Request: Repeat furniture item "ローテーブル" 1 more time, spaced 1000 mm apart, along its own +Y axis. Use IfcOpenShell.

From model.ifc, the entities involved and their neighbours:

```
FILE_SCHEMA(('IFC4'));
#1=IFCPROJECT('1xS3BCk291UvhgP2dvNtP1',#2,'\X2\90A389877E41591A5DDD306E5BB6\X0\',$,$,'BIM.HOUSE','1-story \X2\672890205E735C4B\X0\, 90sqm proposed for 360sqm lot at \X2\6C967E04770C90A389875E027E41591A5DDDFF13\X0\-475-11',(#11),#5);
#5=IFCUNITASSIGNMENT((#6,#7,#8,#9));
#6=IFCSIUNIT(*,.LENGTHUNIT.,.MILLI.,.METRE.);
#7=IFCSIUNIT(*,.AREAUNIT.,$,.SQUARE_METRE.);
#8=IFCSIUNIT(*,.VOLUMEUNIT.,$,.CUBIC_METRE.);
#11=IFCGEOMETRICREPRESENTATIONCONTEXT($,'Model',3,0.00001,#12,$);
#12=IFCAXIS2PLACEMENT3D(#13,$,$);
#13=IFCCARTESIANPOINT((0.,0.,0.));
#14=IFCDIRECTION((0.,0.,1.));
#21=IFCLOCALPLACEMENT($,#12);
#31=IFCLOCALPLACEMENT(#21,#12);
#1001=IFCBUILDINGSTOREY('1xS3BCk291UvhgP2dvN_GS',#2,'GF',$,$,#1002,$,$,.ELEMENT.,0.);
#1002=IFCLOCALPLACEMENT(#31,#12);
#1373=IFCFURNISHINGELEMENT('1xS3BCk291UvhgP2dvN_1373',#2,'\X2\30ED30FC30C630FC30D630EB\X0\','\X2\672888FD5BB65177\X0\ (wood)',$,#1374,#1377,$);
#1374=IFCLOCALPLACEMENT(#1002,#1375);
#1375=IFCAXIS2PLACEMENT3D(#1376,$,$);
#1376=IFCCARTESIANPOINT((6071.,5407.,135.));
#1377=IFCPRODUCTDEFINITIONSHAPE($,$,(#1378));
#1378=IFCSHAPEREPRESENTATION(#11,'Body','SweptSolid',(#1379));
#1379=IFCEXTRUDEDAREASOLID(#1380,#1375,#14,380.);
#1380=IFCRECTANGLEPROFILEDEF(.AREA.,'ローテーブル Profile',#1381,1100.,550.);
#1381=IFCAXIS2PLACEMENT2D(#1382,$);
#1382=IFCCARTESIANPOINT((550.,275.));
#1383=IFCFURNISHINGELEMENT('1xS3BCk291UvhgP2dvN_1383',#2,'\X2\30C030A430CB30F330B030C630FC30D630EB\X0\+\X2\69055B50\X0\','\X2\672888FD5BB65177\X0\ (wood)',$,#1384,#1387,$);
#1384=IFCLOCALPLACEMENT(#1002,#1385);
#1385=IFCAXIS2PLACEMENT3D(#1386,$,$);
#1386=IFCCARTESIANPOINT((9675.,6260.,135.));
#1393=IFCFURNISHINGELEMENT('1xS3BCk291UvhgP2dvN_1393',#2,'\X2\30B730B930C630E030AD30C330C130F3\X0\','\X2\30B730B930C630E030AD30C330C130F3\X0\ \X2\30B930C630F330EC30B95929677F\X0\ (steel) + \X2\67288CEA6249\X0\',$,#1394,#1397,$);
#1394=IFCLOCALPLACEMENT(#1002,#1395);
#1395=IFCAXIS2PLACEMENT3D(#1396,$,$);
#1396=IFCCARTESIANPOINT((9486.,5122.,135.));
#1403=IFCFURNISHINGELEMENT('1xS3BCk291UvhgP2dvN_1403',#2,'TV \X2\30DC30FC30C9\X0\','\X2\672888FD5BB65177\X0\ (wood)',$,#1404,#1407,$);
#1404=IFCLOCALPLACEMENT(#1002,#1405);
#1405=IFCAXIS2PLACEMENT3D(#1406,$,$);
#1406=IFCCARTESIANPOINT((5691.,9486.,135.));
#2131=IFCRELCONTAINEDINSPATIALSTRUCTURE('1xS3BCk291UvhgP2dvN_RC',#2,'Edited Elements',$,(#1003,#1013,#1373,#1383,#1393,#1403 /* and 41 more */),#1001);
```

```python
import ifcopenshell
import ifcopenshell.api.geometry
import ifcopenshell.api.root
import ifcopenshell.util.element
import ifcopenshell.util.placement
import ifcopenshell.util.unit

model = ifcopenshell.open("model.ifc")
unit_scale = ifcopenshell.util.unit.calculate_unit_scale(model)


def reuse_history(source, copy):
    """copy_class also copies each property set's owner history, people and application; keep the originals."""
    for rel in copy.IsDefinedBy:
        if rel.is_a("IfcRelDefinesByProperties") and (history := rel.RelatingPropertyDefinition.OwnerHistory):
            rel.RelatingPropertyDefinition.OwnerHistory = source.OwnerHistory
            ifcopenshell.util.element.remove_deep2(model, history)


source = model.by_guid("1xS3BCk291UvhgP2dvN_1373")
base = ifcopenshell.util.placement.get_local_placement(source.ObjectPlacement)
step = base[:3, 1] * 1 / unit_scale

for i in range(1, 2):
    copy = ifcopenshell.api.root.copy_class(model, product=source)
    copy.Representation = ifcopenshell.util.element.copy_deep(
        model, source.Representation, exclude=["IfcGeometricRepresentationContext", "IfcRepresentationMap"]
    )
    reuse_history(source, copy)
    matrix = base.copy()
    matrix[:3, 3] += i * step
    print("added at", matrix[:3, 3].round(3) + 0.0)
    ifcopenshell.api.geometry.edit_object_placement(model, product=copy, matrix=matrix, is_si=False)

model.write("model_edited.ifc")
```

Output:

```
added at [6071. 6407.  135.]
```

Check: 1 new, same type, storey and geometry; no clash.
